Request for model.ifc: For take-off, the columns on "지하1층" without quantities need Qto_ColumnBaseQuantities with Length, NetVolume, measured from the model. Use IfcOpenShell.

First a look at what the model holds.

```python
import ifcopenshell
import ifcopenshell.util.element
import ifcopenshell.util.unit

model = ifcopenshell.open("model.ifc")
print(model.schema)
for unit_type in ("LENGTHUNIT", "AREAUNIT", "VOLUMEUNIT"):
    print(unit_type, ifcopenshell.util.unit.calculate_unit_scale(model, unit_type))
storey = next(s for s in model.by_type("IfcBuildingStorey") if s.Name == "지하1층")
columns = [e for e in ifcopenshell.util.element.get_decomposition(storey) if e.is_a("IfcColumn")]
for e in sorted(columns, key=lambda e: e.id()):
    print(e.id(), e.is_a(), e.Name, list(ifcopenshell.util.element.get_psets(e, qtos_only=True)), sep=" | ")
```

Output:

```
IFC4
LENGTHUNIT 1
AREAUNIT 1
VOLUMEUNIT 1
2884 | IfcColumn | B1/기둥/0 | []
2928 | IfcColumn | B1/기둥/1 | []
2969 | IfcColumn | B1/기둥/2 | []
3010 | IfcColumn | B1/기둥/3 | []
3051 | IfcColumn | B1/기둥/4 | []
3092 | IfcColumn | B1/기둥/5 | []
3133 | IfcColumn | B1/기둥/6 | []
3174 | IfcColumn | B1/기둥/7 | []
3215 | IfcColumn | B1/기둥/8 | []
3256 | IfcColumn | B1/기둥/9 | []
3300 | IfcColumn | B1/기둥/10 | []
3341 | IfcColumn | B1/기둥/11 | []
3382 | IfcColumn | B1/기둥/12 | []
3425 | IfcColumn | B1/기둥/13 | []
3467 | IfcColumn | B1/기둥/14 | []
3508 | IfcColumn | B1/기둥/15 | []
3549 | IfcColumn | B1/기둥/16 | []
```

```python
import ifcopenshell
import ifcopenshell.api.pset
import ifcopenshell.geom
import ifcopenshell.util.element
import ifcopenshell.util.shape
import ifcopenshell.util.unit

model = ifcopenshell.open("model.ifc")
unit_scale = ifcopenshell.util.unit.calculate_unit_scale(model)
volume_scale = ifcopenshell.util.unit.calculate_unit_scale(model, "VOLUMEUNIT")
settings = ifcopenshell.geom.settings()

storey = next(s for s in model.by_type("IfcBuildingStorey") if s.Name == "지하1층")
columns = [e for e in ifcopenshell.util.element.get_decomposition(storey) if e.is_a("IfcColumn")]

for e in sorted(columns, key=lambda e: e.id()):
    if ifcopenshell.util.element.get_psets(e, qtos_only=True, should_inherit=False):
        continue
    # Geometry comes back in metres, in the element's own axes.
    shape = ifcopenshell.geom.create_shape(settings, e)
    values = {
        "Length": ifcopenshell.util.shape.get_z(shape.geometry) / unit_scale,
        "NetVolume": ifcopenshell.util.shape.get_volume(shape.geometry) / volume_scale,
    }
    qto = ifcopenshell.api.pset.add_qto(model, product=e, name="Qto_ColumnBaseQuantities")
    ifcopenshell.api.pset.edit_qto(model, qto=qto, properties=values)
    print(e.id(), {k: round(v, 3) for k, v in values.items()})

model.write("model-out.ifc")
```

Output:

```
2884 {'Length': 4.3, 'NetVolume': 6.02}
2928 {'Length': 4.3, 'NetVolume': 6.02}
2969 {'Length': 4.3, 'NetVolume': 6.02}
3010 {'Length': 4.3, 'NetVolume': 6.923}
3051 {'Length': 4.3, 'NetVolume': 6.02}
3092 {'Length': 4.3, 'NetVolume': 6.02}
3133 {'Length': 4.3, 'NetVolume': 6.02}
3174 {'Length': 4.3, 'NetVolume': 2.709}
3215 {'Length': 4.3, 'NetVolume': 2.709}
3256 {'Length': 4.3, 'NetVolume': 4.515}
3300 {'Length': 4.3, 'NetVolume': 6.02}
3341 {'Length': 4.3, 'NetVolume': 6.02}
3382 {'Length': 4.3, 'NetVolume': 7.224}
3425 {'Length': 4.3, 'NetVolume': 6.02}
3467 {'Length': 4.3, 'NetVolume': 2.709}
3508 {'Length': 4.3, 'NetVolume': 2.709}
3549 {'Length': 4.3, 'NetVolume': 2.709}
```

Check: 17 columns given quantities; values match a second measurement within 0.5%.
